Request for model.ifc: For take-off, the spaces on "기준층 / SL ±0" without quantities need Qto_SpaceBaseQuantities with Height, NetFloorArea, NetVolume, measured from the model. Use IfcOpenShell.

First a look at what the model holds.

```python
import ifcopenshell
import ifcopenshell.util.element
import ifcopenshell.util.unit

model = ifcopenshell.open("model.ifc")
print(model.schema)
for unit_type in ("LENGTHUNIT", "AREAUNIT", "VOLUMEUNIT"):
    print(unit_type, ifcopenshell.util.unit.calculate_unit_scale(model, unit_type))
storey = next(s for s in model.by_type("IfcBuildingStorey") if s.Name == "기준층 / SL ±0")
spaces = [e for e in ifcopenshell.util.element.get_decomposition(storey) if e.is_a("IfcSpace")]
for e in sorted(spaces, key=lambda e: e.id()):
    print(e.id(), e.is_a(), e.Name, list(ifcopenshell.util.element.get_psets(e, qtos_only=True)), sep=" | ")
```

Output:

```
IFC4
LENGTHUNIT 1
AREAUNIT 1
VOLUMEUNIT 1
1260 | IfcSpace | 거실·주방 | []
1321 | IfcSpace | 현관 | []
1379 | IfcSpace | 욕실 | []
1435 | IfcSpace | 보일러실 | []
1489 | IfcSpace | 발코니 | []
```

```python
import ifcopenshell
import ifcopenshell.api.pset
import ifcopenshell.geom
import ifcopenshell.util.element
import ifcopenshell.util.shape
import ifcopenshell.util.unit

model = ifcopenshell.open("model.ifc")
unit_scale = ifcopenshell.util.unit.calculate_unit_scale(model)
area_scale = ifcopenshell.util.unit.calculate_unit_scale(model, "AREAUNIT")
volume_scale = ifcopenshell.util.unit.calculate_unit_scale(model, "VOLUMEUNIT")
settings = ifcopenshell.geom.settings()

storey = next(s for s in model.by_type("IfcBuildingStorey") if s.Name == "기준층 / SL ±0")
spaces = [e for e in ifcopenshell.util.element.get_decomposition(storey) if e.is_a("IfcSpace")]

for e in sorted(spaces, key=lambda e: e.id()):
    if ifcopenshell.util.element.get_psets(e, qtos_only=True, should_inherit=False):
        continue
    # Geometry comes back in metres, in the element's own axes.
    shape = ifcopenshell.geom.create_shape(settings, e)
    values = {
        "Height": ifcopenshell.util.shape.get_z(shape.geometry) / unit_scale,
        "NetFloorArea": ifcopenshell.util.shape.get_footprint_area(shape.geometry) / area_scale,
        "NetVolume": ifcopenshell.util.shape.get_volume(shape.geometry) / volume_scale,
    }
    qto = ifcopenshell.api.pset.add_qto(model, product=e, name="Qto_SpaceBaseQuantities")
    ifcopenshell.api.pset.edit_qto(model, qto=qto, properties=values)
    print(e.id(), {k: round(v, 3) for k, v in values.items()})

model.write("model_rev.ifc")
```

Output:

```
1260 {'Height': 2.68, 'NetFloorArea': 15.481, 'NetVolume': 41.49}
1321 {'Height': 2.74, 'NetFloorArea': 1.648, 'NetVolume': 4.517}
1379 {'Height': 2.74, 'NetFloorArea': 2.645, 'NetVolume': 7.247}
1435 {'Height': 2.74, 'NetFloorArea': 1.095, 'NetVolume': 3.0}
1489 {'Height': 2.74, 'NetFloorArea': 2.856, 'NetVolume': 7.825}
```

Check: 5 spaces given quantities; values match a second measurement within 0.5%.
